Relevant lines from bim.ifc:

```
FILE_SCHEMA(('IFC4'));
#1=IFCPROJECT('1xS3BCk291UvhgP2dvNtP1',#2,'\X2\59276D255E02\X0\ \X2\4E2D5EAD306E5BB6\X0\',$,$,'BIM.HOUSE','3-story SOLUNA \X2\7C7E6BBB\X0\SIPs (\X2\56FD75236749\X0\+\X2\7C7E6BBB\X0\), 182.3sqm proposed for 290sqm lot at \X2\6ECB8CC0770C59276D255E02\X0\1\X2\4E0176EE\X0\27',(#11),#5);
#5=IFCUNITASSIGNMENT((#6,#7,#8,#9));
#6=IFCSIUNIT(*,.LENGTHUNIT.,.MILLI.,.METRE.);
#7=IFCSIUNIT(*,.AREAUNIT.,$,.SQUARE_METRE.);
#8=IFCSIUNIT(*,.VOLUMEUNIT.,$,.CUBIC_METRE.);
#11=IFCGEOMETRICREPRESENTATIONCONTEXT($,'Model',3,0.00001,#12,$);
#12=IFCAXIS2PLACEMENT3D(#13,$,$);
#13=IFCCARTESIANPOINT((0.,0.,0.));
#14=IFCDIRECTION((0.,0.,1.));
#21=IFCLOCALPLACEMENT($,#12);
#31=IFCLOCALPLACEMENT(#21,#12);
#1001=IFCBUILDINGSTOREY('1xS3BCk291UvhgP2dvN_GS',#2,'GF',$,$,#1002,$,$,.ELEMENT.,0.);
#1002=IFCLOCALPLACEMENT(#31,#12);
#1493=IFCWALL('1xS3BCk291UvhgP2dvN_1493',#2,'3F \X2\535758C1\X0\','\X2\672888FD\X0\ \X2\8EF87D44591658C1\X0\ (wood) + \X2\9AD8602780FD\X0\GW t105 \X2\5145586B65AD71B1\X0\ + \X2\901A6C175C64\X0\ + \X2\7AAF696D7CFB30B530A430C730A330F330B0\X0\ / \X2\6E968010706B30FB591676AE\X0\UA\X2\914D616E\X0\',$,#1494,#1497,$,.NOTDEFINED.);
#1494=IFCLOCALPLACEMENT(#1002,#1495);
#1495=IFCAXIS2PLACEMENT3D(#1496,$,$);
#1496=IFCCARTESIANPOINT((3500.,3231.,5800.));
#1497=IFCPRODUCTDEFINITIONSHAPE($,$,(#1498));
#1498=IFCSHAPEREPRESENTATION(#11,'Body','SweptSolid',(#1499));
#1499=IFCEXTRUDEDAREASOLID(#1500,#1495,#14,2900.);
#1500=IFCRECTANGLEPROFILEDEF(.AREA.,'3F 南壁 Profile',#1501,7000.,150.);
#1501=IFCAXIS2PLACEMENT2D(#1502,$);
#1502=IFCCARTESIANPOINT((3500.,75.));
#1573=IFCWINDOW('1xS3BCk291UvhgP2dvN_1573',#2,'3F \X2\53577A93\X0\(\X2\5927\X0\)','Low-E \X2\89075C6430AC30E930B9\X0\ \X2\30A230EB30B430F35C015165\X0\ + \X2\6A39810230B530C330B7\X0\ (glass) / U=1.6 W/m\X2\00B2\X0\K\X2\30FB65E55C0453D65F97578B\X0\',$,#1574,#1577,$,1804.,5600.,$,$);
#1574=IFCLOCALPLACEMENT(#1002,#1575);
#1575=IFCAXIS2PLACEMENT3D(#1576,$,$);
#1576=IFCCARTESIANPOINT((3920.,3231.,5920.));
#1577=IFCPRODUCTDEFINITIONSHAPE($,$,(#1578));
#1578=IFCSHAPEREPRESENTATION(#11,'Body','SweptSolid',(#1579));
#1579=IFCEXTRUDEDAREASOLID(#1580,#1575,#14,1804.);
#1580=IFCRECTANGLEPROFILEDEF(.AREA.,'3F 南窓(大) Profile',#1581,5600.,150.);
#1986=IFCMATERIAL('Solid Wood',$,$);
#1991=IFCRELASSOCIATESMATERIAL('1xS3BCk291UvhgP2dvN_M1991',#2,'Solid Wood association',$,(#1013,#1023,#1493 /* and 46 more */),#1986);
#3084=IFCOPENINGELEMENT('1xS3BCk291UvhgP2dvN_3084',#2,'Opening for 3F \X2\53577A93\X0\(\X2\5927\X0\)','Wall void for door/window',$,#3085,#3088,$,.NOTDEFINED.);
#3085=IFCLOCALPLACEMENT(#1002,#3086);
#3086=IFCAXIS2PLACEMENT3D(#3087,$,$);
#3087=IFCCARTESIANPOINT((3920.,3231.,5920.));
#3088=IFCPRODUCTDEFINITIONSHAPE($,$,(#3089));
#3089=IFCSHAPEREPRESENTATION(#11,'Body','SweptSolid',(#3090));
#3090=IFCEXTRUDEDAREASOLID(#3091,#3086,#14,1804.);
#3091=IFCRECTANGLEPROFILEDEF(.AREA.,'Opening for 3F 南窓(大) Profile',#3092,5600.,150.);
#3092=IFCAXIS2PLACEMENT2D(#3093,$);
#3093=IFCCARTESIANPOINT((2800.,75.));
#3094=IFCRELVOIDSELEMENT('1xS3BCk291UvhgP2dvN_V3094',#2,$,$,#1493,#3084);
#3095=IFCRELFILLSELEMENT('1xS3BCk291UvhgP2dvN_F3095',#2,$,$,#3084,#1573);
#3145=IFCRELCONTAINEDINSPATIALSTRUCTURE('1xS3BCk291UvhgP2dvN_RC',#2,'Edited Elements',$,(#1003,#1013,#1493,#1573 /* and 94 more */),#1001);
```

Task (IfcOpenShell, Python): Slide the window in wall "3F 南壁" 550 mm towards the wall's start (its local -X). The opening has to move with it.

```python
import ifcopenshell
import ifcopenshell.api.geometry
import ifcopenshell.util.placement

model = ifcopenshell.open("bim.ifc")

window = model.by_id(1573)
opening = window.FillsVoids[0].RelatingOpeningElement
wall = opening.VoidsElements[0].RelatingBuildingElement

wall_matrix = ifcopenshell.util.placement.get_local_placement(wall.ObjectPlacement)
shift = wall_matrix[:3, 0] * -550.0
before = ifcopenshell.util.placement.get_local_placement(window.ObjectPlacement)[:3, 3].copy()

# The window is not placed relative to its opening, so move both.
for product in (opening, window):
    matrix = ifcopenshell.util.placement.get_local_placement(product.ObjectPlacement)
    matrix[:3, 3] += shift
    ifcopenshell.api.geometry.edit_object_placement(model, product=product, matrix=matrix, is_si=False)

after = ifcopenshell.util.placement.get_local_placement(window.ObjectPlacement)[:3, 3]
print("window moved by", (after - before).round(3) + 0.0)

model.write("bim_edited.ifc")
```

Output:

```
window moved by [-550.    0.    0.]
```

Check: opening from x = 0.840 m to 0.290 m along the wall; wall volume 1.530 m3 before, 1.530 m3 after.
